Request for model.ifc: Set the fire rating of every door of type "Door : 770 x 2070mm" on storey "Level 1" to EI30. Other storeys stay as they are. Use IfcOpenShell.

First a look at what the model holds.

```python
import ifcopenshell
import ifcopenshell.util.element

model = ifcopenshell.open("model.ifc")
print(model.schema)
storey = next(s for s in model.by_type("IfcBuildingStorey") if s.Name == "Level 1")
doors = [e for e in ifcopenshell.util.element.get_decomposition(storey) if e.is_a("IfcDoor")]
seen = {}
for e in doors:
    element_type = ifcopenshell.util.element.get_type(e)
    key = (element_type.Name if element_type != e and element_type else None, ifcopenshell.util.element.get_pset(e, "Pset_DoorCommon", "FireRating"))
    seen[key] = seen.get(key, 0) + 1
for (name, value), count in sorted(seen.items(), key=str):
    print(count, "x", name, "|", value)
```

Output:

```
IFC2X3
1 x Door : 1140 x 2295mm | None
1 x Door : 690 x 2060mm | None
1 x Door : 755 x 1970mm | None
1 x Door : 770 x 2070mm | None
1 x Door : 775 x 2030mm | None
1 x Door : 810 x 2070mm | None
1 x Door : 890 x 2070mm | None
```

```python
import ifcopenshell
import ifcopenshell.api.pset
import ifcopenshell.util.element

model = ifcopenshell.open("model.ifc")

storey = next(s for s in model.by_type("IfcBuildingStorey") if s.Name == "Level 1")
doors = [e for e in ifcopenshell.util.element.get_decomposition(storey) if e.is_a("IfcDoor")]

count = 0
for e in doors:
    element_type = ifcopenshell.util.element.get_type(e)
    if element_type in (None, e) or element_type.Name != "Door : 770 x 2070mm":
        continue
    # add_pset returns the element's existing set when there is one.
    pset = ifcopenshell.api.pset.add_pset(model, product=e, name="Pset_DoorCommon")
    ifcopenshell.api.pset.edit_pset(model, pset=pset, properties={"FireRating": "EI30"})
    count += 1

print(count, "doors updated")

model.write("model_updated.ifc")
```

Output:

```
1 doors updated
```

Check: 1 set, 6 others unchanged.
